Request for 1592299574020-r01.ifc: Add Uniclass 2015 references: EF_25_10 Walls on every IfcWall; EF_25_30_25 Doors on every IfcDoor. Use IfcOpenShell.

First a look at what the model holds.

```python
import ifcopenshell

model = ifcopenshell.open("1592299574020-r01.ifc")
print(model.schema)
print("classifications:", [c.Name for c in model.by_type("IfcClassification")])
for ifc_class in ("IfcDoor", "IfcRoof", "IfcStair", "IfcWall", "IfcWindow"):
    print(ifc_class, len(model.by_type(ifc_class)))
```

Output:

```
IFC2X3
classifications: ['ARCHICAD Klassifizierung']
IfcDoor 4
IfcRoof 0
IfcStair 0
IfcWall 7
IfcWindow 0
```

```python
import ifcopenshell
import ifcopenshell.api.classification

model = ifcopenshell.open("1592299574020-r01.ifc")

# IFC2X3 requires Source and Edition and has no link from the project to the system.
system = model.create_entity("IfcClassification", Source="NBS", Edition="2015", Name="Uniclass 2015")

codes = {
    "IfcWall": ("EF_25_10", "Walls"),
    "IfcDoor": ("EF_25_30_25", "Doors"),
}
for ifc_class, (code, name) in codes.items():
    products = model.by_type(ifc_class)
    ifcopenshell.api.classification.add_reference(
        model, products=products, classification=system, identification=code, name=name
    )
    print(code, len(products))

model.write("1592299574020-r01_v2.ifc")
```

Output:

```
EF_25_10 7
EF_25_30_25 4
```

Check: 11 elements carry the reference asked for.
